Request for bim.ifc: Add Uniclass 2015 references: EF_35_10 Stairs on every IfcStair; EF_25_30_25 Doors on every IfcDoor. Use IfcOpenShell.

First a look at what the model holds.

```python
import ifcopenshell

model = ifcopenshell.open("bim.ifc")
print(model.schema)
print("classifications:", [c.Name for c in model.by_type("IfcClassification")])
for ifc_class in ("IfcDoor", "IfcRoof", "IfcStair", "IfcWall", "IfcWindow"):
    print(ifc_class, len(model.by_type(ifc_class)))
```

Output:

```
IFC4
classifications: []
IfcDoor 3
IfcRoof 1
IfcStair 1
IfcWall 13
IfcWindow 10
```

```python
import ifcopenshell
import ifcopenshell.api.classification

model = ifcopenshell.open("bim.ifc")

system = ifcopenshell.api.classification.add_classification(model, classification="Uniclass 2015")

codes = {
    "IfcStair": ("EF_35_10", "Stairs"),
    "IfcDoor": ("EF_25_30_25", "Doors"),
}
for ifc_class, (code, name) in codes.items():
    products = model.by_type(ifc_class)
    ifcopenshell.api.classification.add_reference(
        model, products=products, classification=system, identification=code, name=name
    )
    print(code, len(products))

model.write("bim-out.ifc")
```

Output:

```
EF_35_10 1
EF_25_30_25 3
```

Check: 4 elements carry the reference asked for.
